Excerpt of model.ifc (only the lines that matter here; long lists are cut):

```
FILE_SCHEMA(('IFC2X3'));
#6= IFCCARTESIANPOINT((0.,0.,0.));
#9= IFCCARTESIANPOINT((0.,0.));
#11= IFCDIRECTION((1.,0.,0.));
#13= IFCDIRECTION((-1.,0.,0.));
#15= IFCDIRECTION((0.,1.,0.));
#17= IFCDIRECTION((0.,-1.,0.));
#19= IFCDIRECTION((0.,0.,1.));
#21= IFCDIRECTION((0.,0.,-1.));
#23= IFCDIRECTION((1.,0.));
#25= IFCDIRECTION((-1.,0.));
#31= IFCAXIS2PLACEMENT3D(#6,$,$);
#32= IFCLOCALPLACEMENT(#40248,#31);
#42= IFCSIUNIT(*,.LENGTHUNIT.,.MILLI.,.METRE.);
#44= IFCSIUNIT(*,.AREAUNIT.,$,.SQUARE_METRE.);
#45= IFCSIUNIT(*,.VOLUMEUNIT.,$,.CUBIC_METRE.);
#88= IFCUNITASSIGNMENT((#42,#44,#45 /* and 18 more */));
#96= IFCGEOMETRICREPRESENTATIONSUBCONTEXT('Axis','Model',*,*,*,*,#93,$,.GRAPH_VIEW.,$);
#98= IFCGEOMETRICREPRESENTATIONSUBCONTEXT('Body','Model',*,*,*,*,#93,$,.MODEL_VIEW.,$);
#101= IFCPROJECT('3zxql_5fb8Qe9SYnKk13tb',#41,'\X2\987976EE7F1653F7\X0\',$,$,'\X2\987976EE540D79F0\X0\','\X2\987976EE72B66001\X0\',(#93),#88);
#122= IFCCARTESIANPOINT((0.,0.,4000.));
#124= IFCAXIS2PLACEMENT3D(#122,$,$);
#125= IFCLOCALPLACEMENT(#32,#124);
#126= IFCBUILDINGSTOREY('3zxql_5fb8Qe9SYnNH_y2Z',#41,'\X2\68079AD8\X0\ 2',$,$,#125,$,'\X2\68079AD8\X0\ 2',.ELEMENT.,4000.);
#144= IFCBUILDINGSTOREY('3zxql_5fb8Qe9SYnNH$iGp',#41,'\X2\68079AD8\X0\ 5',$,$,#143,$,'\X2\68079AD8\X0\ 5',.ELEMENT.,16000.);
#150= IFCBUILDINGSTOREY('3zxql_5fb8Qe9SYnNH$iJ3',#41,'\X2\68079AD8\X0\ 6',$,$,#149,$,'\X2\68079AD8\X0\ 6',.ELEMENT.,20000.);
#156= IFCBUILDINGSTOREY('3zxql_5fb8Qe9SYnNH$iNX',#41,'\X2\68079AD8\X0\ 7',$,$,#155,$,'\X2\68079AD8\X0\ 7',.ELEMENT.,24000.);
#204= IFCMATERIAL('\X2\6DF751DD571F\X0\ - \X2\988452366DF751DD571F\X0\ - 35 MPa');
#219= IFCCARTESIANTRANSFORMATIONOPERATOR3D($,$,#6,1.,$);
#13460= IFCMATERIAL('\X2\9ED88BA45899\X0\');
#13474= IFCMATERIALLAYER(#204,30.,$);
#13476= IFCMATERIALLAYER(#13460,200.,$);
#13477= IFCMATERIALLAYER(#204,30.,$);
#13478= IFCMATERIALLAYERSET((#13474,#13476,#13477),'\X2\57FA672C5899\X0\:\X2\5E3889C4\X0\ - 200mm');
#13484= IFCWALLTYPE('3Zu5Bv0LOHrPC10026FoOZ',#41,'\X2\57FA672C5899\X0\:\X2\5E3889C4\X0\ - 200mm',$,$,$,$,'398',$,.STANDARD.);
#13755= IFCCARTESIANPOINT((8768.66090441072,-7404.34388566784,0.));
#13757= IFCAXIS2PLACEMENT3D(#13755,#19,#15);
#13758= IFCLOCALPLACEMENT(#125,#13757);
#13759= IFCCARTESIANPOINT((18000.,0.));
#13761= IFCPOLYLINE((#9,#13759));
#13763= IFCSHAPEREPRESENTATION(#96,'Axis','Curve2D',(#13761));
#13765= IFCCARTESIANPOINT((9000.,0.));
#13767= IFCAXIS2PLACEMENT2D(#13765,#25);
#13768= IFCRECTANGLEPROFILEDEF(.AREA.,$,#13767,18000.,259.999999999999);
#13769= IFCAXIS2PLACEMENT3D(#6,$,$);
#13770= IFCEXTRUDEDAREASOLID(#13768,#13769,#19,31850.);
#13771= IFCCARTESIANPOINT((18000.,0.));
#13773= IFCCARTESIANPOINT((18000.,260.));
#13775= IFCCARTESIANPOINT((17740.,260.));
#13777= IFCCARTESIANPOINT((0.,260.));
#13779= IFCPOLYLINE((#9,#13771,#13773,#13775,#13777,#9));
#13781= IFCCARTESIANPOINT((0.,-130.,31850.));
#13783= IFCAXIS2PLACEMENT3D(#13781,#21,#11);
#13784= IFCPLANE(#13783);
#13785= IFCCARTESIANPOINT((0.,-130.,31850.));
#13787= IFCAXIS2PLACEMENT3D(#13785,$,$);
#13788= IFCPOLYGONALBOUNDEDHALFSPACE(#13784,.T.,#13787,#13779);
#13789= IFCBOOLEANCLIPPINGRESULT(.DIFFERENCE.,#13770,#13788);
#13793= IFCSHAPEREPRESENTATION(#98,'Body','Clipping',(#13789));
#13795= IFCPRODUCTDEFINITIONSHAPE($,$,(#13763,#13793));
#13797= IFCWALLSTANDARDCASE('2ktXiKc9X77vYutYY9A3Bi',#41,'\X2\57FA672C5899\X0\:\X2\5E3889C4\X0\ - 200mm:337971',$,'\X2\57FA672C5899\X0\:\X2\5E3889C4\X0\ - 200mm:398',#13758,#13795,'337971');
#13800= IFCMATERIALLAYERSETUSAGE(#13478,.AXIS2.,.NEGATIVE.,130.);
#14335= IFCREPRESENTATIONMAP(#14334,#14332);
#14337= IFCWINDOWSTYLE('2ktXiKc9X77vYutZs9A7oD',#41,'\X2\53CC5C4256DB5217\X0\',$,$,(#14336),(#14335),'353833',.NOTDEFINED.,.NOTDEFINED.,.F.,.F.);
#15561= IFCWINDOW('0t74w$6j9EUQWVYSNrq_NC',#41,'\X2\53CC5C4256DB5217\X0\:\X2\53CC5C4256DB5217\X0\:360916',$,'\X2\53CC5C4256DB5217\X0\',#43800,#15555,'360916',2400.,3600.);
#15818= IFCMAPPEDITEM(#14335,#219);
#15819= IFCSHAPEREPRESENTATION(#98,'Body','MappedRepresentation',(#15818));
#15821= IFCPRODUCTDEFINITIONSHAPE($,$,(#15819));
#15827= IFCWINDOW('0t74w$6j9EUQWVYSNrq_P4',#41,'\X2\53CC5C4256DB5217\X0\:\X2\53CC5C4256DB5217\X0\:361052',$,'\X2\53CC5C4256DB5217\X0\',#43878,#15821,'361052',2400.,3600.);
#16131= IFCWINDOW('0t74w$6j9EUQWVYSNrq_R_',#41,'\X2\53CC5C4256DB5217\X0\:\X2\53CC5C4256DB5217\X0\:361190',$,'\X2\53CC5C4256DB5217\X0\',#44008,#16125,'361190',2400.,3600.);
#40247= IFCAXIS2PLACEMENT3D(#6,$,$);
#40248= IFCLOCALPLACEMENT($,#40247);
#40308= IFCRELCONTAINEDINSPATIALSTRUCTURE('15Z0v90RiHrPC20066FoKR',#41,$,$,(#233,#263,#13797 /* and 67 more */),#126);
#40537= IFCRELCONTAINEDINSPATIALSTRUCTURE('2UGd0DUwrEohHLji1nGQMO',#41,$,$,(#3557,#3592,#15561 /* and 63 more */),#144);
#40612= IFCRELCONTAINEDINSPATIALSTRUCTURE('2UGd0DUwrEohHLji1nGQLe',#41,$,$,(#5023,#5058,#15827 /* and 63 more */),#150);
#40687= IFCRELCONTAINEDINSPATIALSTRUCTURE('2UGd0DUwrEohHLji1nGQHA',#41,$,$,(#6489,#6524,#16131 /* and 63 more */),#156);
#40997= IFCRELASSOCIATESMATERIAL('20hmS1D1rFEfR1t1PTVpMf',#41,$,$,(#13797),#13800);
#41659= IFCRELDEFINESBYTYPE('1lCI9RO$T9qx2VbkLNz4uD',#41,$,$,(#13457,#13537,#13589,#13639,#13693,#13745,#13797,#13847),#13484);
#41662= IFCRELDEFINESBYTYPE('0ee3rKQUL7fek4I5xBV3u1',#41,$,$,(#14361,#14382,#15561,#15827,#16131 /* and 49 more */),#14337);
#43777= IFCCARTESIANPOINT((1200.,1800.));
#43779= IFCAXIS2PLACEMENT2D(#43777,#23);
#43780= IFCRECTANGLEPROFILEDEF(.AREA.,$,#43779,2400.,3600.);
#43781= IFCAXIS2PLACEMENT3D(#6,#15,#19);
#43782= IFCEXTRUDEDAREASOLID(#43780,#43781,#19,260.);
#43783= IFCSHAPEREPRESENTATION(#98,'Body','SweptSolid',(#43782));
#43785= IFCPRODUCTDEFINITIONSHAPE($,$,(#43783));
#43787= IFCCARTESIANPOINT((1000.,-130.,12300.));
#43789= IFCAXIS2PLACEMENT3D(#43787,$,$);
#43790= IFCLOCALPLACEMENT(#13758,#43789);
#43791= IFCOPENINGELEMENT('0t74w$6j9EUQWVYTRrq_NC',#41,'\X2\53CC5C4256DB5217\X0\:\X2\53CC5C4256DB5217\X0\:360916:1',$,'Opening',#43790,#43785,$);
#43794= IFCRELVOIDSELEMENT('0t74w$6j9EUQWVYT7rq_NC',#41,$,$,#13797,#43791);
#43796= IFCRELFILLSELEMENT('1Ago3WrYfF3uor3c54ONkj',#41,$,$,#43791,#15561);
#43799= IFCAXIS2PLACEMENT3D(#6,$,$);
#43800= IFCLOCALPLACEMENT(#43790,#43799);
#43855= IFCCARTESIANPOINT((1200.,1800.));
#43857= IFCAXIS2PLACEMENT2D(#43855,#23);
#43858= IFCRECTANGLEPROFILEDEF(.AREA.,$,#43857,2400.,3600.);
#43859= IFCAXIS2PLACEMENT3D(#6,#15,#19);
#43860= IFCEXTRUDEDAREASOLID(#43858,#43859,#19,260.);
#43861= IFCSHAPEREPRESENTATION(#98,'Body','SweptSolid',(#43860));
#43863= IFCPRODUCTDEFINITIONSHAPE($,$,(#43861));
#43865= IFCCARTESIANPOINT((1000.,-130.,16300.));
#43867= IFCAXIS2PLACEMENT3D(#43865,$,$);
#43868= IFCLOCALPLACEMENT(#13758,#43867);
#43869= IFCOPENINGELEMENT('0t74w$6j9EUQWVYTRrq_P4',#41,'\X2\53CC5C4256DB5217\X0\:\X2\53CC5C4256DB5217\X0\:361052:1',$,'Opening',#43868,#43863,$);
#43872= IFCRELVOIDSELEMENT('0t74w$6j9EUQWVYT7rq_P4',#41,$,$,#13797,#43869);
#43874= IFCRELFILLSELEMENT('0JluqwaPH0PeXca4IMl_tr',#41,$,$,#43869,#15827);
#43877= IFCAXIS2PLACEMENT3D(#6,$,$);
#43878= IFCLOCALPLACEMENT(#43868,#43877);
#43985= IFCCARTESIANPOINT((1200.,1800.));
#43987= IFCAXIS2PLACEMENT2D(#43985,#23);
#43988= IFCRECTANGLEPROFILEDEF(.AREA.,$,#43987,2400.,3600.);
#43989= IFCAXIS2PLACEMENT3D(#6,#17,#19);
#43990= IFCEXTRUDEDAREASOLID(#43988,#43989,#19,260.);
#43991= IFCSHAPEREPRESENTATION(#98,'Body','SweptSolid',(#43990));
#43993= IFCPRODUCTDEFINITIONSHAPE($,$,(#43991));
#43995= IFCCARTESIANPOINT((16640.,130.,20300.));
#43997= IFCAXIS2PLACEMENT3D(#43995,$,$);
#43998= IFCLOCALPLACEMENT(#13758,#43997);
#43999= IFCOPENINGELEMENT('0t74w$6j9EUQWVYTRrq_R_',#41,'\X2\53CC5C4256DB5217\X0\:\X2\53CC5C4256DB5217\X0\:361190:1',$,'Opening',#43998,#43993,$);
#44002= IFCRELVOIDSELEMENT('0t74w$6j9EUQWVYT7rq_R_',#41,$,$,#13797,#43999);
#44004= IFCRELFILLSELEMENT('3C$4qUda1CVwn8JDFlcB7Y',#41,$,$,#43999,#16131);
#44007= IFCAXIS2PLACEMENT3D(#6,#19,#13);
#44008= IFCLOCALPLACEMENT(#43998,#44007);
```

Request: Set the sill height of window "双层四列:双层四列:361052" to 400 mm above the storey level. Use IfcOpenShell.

```python
import numpy as np
import ifcopenshell
import ifcopenshell.api.geometry
import ifcopenshell.geom
import ifcopenshell.util.element
import ifcopenshell.util.placement
import ifcopenshell.util.shape
import ifcopenshell.util.unit

model = ifcopenshell.open("model.ifc")
unit_scale = ifcopenshell.util.unit.calculate_unit_scale(model)

window = model.by_guid("0t74w$6j9EUQWVYSNrq_P4")
opening = window.FillsVoids[0].RelatingOpeningElement
storey = ifcopenshell.util.element.get_container(window, ifc_class="IfcBuildingStorey")
level = ifcopenshell.util.placement.get_local_placement(storey.ObjectPlacement)[2, 3]

# The opening's origin need not be at the sill, so measure its lowest point.
shape = ifcopenshell.geom.create_shape(ifcopenshell.geom.settings(), opening)
bottom = ifcopenshell.util.shape.get_shape_bottom_elevation(shape, shape.geometry) / unit_scale
dz = level + 400.0 - bottom

shift = np.array([0.0, 0.0, dz])
# The window is placed relative to its opening, so it follows when the opening moves.
matrix = ifcopenshell.util.placement.get_local_placement(opening.ObjectPlacement)
matrix[:3, 3] += shift
ifcopenshell.api.geometry.edit_object_placement(
    model, product=opening, matrix=matrix, is_si=False, should_transform_children=True
)

print(f"moved by {dz * unit_scale:+.3f} m")

model.write("model_rev.ifc")
```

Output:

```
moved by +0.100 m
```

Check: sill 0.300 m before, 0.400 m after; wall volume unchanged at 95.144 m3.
